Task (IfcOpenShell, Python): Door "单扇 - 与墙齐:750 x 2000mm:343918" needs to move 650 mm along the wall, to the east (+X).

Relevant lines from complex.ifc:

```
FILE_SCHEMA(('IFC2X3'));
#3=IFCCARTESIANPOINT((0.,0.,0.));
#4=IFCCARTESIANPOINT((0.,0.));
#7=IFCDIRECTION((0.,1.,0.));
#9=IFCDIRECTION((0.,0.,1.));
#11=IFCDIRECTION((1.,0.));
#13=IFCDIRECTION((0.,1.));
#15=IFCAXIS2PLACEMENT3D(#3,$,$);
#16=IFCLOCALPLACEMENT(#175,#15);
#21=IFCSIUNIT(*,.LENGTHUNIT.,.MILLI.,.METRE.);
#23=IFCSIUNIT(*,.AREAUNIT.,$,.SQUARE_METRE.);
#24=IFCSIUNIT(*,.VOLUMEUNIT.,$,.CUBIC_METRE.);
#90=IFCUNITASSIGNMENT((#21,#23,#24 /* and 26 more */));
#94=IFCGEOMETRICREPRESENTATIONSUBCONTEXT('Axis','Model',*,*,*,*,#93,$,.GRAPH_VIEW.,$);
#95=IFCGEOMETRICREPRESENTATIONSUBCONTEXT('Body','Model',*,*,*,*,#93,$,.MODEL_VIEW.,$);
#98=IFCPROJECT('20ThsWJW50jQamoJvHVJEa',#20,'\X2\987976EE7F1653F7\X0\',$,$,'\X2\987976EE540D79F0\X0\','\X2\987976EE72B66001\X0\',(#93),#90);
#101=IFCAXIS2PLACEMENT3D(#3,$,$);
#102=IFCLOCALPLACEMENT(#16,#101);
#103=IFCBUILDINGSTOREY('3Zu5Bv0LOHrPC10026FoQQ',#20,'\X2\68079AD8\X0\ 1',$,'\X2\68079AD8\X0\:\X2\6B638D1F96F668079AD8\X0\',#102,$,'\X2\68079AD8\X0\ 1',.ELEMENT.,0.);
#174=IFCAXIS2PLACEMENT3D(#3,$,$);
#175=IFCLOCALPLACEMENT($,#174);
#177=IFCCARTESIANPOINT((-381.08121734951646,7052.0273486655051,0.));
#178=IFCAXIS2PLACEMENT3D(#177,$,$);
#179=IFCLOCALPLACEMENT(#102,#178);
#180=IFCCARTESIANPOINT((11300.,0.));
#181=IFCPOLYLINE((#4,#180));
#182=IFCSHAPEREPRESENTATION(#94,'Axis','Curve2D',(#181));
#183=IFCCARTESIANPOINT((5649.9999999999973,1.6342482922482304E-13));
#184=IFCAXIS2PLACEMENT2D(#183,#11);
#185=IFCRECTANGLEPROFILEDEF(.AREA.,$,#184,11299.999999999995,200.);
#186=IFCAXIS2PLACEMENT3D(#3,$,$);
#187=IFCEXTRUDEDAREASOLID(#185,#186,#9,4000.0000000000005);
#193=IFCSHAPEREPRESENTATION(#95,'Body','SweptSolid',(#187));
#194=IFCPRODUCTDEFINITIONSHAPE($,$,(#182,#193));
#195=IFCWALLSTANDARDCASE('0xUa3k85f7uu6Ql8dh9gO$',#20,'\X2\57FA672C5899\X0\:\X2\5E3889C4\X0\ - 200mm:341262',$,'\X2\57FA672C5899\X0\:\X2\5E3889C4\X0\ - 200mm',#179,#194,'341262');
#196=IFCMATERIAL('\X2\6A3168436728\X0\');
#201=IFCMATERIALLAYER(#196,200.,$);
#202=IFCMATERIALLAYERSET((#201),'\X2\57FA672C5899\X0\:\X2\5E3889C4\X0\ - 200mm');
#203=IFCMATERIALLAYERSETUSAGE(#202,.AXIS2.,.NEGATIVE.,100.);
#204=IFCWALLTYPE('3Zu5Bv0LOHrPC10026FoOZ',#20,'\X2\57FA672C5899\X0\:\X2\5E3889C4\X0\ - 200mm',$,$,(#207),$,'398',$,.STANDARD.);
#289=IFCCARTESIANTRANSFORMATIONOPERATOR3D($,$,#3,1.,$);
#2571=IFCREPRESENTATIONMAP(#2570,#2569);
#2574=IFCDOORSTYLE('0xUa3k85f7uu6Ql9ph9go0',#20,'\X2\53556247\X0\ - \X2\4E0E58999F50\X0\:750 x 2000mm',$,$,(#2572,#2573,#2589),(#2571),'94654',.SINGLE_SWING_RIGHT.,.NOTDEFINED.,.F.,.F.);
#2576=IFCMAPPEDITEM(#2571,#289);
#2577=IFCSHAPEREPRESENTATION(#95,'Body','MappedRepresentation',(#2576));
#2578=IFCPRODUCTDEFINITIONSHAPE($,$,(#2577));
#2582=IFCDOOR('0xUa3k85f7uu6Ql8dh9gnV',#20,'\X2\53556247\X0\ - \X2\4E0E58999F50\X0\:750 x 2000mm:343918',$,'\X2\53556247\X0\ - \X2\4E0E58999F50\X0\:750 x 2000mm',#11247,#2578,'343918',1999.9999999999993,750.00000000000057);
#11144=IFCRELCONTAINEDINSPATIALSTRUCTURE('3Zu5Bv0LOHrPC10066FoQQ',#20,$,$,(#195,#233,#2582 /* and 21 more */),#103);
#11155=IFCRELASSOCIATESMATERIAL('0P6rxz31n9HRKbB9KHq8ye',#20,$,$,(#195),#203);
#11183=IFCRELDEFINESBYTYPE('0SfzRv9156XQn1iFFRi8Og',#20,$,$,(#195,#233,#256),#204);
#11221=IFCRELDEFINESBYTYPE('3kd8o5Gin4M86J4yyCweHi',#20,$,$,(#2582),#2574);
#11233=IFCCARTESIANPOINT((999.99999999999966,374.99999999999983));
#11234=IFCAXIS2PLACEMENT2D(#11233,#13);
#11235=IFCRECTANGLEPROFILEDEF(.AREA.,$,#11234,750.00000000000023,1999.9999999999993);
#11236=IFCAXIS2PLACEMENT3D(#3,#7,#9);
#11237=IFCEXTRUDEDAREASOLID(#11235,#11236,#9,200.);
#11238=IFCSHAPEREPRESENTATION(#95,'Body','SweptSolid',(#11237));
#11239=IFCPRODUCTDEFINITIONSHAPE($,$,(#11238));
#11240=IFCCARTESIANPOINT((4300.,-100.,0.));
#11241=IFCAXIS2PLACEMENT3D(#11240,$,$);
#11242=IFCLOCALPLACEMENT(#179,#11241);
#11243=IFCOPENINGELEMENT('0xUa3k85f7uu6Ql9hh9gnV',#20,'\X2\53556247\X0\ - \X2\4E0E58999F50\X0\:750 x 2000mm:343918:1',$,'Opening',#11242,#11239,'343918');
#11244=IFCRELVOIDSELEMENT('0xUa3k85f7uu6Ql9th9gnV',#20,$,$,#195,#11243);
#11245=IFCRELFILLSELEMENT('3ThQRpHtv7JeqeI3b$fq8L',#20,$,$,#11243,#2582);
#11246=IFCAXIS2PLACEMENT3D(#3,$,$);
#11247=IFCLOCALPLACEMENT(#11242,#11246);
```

```python
import ifcopenshell
import ifcopenshell.api.geometry
import ifcopenshell.util.placement

model = ifcopenshell.open("complex.ifc")

door = model.by_guid("0xUa3k85f7uu6Ql8dh9gnV")
opening = door.FillsVoids[0].RelatingOpeningElement
wall = opening.VoidsElements[0].RelatingBuildingElement

wall_matrix = ifcopenshell.util.placement.get_local_placement(wall.ObjectPlacement)
shift = wall_matrix[:3, 0] * 650.0
before = ifcopenshell.util.placement.get_local_placement(door.ObjectPlacement)[:3, 3].copy()

# The door is placed relative to its opening, so it follows when the opening moves.
matrix = ifcopenshell.util.placement.get_local_placement(opening.ObjectPlacement)
matrix[:3, 3] += shift
ifcopenshell.api.geometry.edit_object_placement(
    model, product=opening, matrix=matrix, is_si=False, should_transform_children=True
)

after = ifcopenshell.util.placement.get_local_placement(door.ObjectPlacement)[:3, 3]
print("door moved by", (after - before).round(3) + 0.0)

model.write("complex-out.ifc")
```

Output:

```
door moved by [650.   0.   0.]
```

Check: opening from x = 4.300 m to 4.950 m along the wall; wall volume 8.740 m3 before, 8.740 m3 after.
